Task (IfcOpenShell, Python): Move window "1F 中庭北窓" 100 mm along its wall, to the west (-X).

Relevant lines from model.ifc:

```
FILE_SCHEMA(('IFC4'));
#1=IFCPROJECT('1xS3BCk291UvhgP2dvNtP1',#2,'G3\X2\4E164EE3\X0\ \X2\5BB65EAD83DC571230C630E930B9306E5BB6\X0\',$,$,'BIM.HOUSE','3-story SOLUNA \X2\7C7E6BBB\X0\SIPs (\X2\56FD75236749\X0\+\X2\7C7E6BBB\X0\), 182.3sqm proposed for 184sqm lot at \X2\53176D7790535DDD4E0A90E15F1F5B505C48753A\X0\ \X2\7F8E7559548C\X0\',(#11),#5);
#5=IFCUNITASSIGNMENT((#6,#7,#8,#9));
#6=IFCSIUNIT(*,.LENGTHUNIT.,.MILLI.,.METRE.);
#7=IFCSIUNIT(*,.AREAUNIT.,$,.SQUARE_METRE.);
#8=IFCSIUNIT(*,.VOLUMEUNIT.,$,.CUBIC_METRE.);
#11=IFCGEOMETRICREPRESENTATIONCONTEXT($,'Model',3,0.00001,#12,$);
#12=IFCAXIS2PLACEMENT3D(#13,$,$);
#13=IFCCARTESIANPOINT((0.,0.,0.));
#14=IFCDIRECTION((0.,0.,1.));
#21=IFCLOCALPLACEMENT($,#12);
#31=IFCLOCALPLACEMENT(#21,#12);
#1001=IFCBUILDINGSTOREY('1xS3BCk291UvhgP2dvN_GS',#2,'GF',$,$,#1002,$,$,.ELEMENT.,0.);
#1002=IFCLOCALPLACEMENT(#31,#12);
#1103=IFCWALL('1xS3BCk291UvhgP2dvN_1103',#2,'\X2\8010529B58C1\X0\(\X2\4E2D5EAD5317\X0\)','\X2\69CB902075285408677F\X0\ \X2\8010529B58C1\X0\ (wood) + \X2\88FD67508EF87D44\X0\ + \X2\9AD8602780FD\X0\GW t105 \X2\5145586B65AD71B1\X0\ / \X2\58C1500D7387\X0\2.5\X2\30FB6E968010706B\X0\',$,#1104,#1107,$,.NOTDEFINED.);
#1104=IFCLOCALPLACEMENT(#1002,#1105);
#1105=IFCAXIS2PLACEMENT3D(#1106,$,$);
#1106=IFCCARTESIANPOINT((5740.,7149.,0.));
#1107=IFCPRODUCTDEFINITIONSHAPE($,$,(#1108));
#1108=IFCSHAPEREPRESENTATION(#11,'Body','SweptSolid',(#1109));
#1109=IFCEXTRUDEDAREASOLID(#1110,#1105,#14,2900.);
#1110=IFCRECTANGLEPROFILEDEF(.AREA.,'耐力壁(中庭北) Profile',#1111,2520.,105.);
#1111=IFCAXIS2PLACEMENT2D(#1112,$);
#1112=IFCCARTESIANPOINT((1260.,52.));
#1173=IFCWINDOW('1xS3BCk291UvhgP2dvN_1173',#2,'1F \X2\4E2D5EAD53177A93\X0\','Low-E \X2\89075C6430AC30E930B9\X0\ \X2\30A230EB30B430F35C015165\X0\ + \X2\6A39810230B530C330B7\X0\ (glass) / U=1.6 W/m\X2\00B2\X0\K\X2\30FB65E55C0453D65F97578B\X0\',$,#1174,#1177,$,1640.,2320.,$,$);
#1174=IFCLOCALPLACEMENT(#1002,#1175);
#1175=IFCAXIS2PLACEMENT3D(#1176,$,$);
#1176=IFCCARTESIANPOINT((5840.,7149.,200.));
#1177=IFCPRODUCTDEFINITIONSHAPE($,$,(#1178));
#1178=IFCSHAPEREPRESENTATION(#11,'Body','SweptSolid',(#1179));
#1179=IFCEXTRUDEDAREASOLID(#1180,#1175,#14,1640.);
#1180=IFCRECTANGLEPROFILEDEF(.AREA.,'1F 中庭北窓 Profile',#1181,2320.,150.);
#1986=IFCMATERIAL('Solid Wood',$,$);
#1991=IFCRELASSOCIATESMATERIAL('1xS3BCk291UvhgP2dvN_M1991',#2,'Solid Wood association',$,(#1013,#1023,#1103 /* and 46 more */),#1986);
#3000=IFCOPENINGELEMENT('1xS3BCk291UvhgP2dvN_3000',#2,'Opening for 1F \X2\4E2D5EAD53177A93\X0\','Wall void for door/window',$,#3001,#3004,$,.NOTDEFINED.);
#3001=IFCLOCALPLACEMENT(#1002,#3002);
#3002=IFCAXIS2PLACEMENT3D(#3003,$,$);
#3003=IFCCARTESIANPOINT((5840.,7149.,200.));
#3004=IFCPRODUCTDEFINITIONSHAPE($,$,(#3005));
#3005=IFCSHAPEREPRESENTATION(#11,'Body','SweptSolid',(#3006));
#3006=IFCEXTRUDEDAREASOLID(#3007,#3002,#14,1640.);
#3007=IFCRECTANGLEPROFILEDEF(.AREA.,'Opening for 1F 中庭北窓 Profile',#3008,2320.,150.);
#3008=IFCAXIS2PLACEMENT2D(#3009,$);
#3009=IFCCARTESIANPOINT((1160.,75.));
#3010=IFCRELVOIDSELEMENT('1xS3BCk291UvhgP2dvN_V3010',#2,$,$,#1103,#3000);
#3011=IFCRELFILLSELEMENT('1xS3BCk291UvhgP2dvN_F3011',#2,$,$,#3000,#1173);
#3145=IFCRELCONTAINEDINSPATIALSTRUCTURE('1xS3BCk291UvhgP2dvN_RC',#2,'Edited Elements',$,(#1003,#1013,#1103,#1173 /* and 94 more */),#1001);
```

```python
import ifcopenshell
import ifcopenshell.api.geometry
import ifcopenshell.util.placement
import ifcopenshell.util.unit

model = ifcopenshell.open("model.ifc")
unit_scale = ifcopenshell.util.unit.calculate_unit_scale(model)

window = model.by_guid("1xS3BCk291UvhgP2dvN_1173")
opening = window.FillsVoids[0].RelatingOpeningElement
wall = opening.VoidsElements[0].RelatingBuildingElement

wall_matrix = ifcopenshell.util.placement.get_local_placement(wall.ObjectPlacement)
shift = wall_matrix[:3, 0] * -0.1 / unit_scale
before = ifcopenshell.util.placement.get_local_placement(window.ObjectPlacement)[:3, 3].copy()

# The window is not placed relative to its opening, so move both.
for product in (opening, window):
    matrix = ifcopenshell.util.placement.get_local_placement(product.ObjectPlacement)
    matrix[:3, 3] += shift
    ifcopenshell.api.geometry.edit_object_placement(model, product=product, matrix=matrix, is_si=False)

after = ifcopenshell.util.placement.get_local_placement(window.ObjectPlacement)[:3, 3]
print("window moved by", (after - before).round(3) + 0.0)

model.write("model_edited.ifc")
```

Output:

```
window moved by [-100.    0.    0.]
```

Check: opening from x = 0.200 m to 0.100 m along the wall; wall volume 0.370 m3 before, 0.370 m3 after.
